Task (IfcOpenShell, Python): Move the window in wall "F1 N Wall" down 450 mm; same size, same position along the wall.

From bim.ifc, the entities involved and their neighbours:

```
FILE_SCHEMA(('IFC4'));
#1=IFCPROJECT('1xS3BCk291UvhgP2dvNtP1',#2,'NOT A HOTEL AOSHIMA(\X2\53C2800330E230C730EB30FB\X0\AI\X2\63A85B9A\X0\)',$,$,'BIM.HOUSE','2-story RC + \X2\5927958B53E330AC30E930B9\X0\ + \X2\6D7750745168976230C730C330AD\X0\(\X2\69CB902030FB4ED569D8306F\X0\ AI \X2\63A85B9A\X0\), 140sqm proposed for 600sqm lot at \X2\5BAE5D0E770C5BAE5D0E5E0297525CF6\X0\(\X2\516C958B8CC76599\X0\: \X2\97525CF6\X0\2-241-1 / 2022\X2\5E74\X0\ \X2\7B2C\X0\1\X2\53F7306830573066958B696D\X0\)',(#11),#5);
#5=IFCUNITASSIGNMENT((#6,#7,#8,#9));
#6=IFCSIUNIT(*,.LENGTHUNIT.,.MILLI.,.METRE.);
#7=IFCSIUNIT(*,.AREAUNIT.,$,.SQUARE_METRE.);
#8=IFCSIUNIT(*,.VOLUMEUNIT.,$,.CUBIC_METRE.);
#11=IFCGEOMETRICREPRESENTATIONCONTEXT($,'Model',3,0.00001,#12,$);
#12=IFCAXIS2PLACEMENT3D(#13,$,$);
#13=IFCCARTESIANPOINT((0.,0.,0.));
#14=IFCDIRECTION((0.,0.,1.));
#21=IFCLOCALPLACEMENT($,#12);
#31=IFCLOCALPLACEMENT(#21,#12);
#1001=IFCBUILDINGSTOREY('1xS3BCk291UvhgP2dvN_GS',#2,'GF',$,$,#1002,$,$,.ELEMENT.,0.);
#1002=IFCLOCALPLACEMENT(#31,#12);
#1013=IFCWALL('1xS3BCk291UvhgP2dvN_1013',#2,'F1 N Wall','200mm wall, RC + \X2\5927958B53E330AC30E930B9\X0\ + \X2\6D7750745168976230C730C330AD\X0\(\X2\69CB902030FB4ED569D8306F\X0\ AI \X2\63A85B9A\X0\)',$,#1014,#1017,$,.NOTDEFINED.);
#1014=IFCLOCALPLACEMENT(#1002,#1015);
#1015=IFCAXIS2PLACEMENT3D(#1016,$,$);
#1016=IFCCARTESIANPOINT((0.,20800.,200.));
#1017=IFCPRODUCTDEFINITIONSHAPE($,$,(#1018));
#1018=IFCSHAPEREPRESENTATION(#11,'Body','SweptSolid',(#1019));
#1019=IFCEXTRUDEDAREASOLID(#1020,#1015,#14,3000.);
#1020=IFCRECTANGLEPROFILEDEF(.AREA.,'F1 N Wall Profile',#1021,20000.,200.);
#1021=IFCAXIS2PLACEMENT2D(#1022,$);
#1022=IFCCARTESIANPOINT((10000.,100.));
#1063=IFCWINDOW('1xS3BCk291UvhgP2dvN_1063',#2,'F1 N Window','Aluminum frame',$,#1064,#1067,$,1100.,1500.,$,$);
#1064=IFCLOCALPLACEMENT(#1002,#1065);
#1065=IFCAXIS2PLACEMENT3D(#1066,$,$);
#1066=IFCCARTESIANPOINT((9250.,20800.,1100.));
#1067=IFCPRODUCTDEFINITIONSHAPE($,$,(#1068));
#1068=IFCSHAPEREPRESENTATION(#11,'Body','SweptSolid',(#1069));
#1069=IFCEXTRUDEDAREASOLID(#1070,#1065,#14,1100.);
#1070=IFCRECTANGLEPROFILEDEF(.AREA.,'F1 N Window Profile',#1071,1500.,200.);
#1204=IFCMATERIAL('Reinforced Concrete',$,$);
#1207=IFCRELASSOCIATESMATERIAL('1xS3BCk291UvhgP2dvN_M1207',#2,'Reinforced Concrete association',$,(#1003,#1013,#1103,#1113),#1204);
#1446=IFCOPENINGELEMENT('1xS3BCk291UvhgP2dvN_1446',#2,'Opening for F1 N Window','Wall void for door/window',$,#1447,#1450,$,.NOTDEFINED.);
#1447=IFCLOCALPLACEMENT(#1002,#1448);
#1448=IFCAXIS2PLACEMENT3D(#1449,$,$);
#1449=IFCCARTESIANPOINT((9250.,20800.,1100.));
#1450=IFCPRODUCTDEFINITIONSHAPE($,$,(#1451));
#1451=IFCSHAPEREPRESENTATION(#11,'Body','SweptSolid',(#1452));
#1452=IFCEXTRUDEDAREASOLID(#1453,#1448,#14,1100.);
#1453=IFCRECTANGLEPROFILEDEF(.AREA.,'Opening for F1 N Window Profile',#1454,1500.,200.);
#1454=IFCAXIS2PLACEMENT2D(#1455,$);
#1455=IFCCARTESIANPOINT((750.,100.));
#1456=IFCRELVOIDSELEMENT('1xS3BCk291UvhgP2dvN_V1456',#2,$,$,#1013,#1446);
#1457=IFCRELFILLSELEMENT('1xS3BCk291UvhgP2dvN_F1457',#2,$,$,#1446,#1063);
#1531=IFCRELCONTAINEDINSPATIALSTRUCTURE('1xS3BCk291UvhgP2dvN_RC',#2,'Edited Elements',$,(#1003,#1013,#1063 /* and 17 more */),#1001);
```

```python
import numpy as np
import ifcopenshell
import ifcopenshell.api.geometry
import ifcopenshell.util.placement
import ifcopenshell.util.unit

model = ifcopenshell.open("bim.ifc")
unit_scale = ifcopenshell.util.unit.calculate_unit_scale(model)

window = model.by_id(1063)
opening = window.FillsVoids[0].RelatingOpeningElement
dz = -0.45 / unit_scale

shift = np.array([0.0, 0.0, dz])
# The window is not placed relative to its opening, so move both.
for product in (opening, window):
    matrix = ifcopenshell.util.placement.get_local_placement(product.ObjectPlacement)
    matrix[:3, 3] += shift
    ifcopenshell.api.geometry.edit_object_placement(model, product=product, matrix=matrix, is_si=False)

print(f"moved by {dz * unit_scale:+.3f} m")

model.write("bim_edited.ifc")
```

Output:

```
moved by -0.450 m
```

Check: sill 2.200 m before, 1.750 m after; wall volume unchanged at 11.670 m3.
